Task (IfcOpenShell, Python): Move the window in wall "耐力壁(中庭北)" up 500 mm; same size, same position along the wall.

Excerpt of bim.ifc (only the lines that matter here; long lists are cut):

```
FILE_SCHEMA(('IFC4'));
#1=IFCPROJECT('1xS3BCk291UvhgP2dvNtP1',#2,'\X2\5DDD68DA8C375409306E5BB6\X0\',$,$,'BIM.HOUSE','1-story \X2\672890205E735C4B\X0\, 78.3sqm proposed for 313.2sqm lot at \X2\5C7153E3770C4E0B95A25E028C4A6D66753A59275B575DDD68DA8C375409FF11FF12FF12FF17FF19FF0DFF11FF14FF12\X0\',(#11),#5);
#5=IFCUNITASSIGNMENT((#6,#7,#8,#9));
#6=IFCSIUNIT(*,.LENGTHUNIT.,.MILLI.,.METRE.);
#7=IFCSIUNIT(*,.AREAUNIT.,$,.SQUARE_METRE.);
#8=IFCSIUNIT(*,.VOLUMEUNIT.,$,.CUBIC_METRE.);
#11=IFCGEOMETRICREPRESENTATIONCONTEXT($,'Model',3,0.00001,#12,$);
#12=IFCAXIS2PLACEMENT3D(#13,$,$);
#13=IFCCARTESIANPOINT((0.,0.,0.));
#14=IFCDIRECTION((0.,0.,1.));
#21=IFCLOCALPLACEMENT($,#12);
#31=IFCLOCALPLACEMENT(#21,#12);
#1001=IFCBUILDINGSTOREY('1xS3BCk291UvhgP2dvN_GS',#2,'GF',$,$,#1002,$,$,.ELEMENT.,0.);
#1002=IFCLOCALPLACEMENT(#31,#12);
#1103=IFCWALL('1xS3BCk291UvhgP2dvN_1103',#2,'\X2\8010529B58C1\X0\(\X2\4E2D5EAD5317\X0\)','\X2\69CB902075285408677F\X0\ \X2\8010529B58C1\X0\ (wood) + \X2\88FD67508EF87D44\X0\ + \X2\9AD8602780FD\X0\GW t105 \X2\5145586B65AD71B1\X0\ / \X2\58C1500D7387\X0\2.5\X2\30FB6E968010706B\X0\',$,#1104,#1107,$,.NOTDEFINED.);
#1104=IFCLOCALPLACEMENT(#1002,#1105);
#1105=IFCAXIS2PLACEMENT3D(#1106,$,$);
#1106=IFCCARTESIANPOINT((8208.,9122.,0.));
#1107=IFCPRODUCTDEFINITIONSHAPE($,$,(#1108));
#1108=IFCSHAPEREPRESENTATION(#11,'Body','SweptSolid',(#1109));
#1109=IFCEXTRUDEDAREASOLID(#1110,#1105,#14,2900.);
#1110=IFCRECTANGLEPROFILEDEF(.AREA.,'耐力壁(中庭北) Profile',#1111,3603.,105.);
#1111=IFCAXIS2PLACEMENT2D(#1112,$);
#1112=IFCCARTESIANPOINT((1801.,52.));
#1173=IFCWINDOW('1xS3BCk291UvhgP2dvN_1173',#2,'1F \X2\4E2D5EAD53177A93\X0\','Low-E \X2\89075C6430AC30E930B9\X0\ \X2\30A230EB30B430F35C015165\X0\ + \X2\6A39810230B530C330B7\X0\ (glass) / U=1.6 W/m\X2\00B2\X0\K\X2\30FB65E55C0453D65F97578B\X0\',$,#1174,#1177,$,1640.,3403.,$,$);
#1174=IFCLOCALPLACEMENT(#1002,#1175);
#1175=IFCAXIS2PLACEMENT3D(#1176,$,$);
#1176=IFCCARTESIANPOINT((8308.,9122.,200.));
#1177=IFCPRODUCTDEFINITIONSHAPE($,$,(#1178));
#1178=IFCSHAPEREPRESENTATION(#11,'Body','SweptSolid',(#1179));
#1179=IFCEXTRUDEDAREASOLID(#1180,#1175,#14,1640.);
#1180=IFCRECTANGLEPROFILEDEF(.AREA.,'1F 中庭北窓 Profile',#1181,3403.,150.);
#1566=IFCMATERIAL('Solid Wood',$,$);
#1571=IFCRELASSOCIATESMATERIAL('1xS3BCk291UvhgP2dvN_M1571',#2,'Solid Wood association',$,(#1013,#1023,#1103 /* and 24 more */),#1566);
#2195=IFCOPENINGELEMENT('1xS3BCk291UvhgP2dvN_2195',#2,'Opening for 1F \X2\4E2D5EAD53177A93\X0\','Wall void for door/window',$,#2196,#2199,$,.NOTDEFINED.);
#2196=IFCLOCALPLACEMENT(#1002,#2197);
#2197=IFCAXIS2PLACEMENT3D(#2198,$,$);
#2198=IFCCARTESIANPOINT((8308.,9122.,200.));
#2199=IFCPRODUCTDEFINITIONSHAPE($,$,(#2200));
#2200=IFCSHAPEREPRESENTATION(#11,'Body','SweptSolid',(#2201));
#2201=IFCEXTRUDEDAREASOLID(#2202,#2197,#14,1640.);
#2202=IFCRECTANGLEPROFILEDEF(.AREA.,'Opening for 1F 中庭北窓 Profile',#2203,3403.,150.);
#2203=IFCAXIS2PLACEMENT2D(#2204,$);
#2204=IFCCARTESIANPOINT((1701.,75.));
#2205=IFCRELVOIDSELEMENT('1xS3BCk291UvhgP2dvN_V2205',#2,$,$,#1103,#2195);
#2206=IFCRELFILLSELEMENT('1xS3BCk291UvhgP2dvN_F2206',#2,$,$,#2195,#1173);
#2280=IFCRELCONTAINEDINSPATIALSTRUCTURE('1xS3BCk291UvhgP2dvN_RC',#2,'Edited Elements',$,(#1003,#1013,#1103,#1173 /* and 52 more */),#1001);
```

```python
import numpy as np
import ifcopenshell
import ifcopenshell.api.geometry
import ifcopenshell.util.placement
import ifcopenshell.util.unit

model = ifcopenshell.open("bim.ifc")
unit_scale = ifcopenshell.util.unit.calculate_unit_scale(model)

window = model.by_id(1173)
opening = window.FillsVoids[0].RelatingOpeningElement
dz = 0.5 / unit_scale

shift = np.array([0.0, 0.0, dz])
# The window is not placed relative to its opening, so move both.
for product in (opening, window):
    matrix = ifcopenshell.util.placement.get_local_placement(product.ObjectPlacement)
    matrix[:3, 3] += shift
    ifcopenshell.api.geometry.edit_object_placement(model, product=product, matrix=matrix, is_si=False)

print(f"moved by {dz * unit_scale:+.3f} m")

model.write("bim-out.ifc")
```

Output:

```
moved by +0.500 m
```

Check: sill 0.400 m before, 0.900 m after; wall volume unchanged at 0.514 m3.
